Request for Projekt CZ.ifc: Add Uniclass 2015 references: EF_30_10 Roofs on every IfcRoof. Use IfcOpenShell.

First a look at what the model holds.

```python
import ifcopenshell

model = ifcopenshell.open("Projekt CZ.ifc")
print(model.schema)
print("classifications:", [c.Name for c in model.by_type("IfcClassification")])
for ifc_class in ("IfcDoor", "IfcRoof", "IfcStair", "IfcWall", "IfcWindow"):
    print(ifc_class, len(model.by_type(ifc_class)))
```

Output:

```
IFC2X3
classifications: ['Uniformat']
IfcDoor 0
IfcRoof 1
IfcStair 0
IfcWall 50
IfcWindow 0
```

```python
import ifcopenshell
import ifcopenshell.api.classification

model = ifcopenshell.open("Projekt CZ.ifc")

# IFC2X3 requires Source and Edition and has no link from the project to the system.
system = model.create_entity("IfcClassification", Source="NBS", Edition="2015", Name="Uniclass 2015")

codes = {
    "IfcRoof": ("EF_30_10", "Roofs"),
}
for ifc_class, (code, name) in codes.items():
    products = model.by_type(ifc_class)
    ifcopenshell.api.classification.add_reference(
        model, products=products, classification=system, identification=code, name=name
    )
    print(code, len(products))

model.write("Projekt CZ_edited.ifc")
```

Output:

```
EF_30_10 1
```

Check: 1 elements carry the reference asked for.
